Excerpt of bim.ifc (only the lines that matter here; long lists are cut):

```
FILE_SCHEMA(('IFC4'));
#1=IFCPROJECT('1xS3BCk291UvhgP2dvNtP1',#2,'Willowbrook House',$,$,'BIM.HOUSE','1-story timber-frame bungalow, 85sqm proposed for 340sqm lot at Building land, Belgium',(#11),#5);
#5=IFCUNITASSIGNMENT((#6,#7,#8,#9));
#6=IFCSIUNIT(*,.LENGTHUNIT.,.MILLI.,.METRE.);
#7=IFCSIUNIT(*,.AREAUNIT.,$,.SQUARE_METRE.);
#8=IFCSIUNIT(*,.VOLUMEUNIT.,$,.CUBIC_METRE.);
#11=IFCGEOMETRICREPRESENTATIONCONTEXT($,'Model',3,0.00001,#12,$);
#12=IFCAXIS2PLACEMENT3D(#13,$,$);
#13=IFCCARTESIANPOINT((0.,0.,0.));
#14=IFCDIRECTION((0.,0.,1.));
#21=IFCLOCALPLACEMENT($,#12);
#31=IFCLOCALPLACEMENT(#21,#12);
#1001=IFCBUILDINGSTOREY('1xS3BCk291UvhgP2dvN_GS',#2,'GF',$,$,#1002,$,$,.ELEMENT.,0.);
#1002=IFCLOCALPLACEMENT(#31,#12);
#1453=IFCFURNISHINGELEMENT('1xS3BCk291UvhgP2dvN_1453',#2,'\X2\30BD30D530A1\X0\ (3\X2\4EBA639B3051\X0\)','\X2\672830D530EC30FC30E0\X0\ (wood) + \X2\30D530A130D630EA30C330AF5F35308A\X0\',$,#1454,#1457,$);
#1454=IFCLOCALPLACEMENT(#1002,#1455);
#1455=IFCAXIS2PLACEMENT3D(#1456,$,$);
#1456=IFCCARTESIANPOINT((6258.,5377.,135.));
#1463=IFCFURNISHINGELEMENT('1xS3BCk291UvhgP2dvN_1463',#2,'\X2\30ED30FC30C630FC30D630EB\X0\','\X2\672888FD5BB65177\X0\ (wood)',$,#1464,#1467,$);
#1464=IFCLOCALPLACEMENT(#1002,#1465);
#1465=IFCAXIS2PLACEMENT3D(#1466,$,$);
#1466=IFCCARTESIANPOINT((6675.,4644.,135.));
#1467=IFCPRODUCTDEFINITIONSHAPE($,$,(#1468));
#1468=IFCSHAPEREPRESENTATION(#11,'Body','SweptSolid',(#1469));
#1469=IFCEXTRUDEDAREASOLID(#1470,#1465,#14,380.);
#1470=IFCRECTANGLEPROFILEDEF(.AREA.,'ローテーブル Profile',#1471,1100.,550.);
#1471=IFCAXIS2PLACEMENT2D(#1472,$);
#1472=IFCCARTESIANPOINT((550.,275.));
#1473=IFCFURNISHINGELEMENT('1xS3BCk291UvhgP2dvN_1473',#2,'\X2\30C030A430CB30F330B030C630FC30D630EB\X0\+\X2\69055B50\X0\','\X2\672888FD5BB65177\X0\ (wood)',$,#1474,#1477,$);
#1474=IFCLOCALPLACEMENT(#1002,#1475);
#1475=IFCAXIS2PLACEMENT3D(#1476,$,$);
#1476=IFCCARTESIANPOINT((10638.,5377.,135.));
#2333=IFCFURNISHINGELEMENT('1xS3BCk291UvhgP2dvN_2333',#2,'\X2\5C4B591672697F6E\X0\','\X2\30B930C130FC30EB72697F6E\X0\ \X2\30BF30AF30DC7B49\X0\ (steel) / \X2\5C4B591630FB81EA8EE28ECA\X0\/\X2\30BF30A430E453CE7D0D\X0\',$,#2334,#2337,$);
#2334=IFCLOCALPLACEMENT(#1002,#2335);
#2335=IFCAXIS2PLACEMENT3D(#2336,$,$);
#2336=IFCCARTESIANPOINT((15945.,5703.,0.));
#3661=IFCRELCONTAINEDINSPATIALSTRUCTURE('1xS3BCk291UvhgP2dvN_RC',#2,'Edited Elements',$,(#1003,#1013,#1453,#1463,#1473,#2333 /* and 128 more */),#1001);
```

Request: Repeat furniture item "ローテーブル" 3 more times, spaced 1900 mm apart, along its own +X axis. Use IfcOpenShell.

```python
import ifcopenshell
import ifcopenshell.api.geometry
import ifcopenshell.api.root
import ifcopenshell.util.element
import ifcopenshell.util.placement
import ifcopenshell.util.unit

model = ifcopenshell.open("bim.ifc")
unit_scale = ifcopenshell.util.unit.calculate_unit_scale(model)


def reuse_history(source, copy):
    """copy_class also copies each property set's owner history, people and application; keep the originals."""
    for rel in copy.IsDefinedBy:
        if rel.is_a("IfcRelDefinesByProperties") and (history := rel.RelatingPropertyDefinition.OwnerHistory):
            rel.RelatingPropertyDefinition.OwnerHistory = source.OwnerHistory
            ifcopenshell.util.element.remove_deep2(model, history)


source = model.by_id(1463)
base = ifcopenshell.util.placement.get_local_placement(source.ObjectPlacement)
step = base[:3, 0] * 1.9 / unit_scale

for i in range(1, 4):
    copy = ifcopenshell.api.root.copy_class(model, product=source)
    copy.Representation = ifcopenshell.util.element.copy_deep(
        model, source.Representation, exclude=["IfcGeometricRepresentationContext", "IfcRepresentationMap"]
    )
    reuse_history(source, copy)
    matrix = base.copy()
    matrix[:3, 3] += i * step
    print("added at", matrix[:3, 3].round(3) + 0.0)
    ifcopenshell.api.geometry.edit_object_placement(model, product=copy, matrix=matrix, is_si=False)

model.write("bim_rev.ifc")
```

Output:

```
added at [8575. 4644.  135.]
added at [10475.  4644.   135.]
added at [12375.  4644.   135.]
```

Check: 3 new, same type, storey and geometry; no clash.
